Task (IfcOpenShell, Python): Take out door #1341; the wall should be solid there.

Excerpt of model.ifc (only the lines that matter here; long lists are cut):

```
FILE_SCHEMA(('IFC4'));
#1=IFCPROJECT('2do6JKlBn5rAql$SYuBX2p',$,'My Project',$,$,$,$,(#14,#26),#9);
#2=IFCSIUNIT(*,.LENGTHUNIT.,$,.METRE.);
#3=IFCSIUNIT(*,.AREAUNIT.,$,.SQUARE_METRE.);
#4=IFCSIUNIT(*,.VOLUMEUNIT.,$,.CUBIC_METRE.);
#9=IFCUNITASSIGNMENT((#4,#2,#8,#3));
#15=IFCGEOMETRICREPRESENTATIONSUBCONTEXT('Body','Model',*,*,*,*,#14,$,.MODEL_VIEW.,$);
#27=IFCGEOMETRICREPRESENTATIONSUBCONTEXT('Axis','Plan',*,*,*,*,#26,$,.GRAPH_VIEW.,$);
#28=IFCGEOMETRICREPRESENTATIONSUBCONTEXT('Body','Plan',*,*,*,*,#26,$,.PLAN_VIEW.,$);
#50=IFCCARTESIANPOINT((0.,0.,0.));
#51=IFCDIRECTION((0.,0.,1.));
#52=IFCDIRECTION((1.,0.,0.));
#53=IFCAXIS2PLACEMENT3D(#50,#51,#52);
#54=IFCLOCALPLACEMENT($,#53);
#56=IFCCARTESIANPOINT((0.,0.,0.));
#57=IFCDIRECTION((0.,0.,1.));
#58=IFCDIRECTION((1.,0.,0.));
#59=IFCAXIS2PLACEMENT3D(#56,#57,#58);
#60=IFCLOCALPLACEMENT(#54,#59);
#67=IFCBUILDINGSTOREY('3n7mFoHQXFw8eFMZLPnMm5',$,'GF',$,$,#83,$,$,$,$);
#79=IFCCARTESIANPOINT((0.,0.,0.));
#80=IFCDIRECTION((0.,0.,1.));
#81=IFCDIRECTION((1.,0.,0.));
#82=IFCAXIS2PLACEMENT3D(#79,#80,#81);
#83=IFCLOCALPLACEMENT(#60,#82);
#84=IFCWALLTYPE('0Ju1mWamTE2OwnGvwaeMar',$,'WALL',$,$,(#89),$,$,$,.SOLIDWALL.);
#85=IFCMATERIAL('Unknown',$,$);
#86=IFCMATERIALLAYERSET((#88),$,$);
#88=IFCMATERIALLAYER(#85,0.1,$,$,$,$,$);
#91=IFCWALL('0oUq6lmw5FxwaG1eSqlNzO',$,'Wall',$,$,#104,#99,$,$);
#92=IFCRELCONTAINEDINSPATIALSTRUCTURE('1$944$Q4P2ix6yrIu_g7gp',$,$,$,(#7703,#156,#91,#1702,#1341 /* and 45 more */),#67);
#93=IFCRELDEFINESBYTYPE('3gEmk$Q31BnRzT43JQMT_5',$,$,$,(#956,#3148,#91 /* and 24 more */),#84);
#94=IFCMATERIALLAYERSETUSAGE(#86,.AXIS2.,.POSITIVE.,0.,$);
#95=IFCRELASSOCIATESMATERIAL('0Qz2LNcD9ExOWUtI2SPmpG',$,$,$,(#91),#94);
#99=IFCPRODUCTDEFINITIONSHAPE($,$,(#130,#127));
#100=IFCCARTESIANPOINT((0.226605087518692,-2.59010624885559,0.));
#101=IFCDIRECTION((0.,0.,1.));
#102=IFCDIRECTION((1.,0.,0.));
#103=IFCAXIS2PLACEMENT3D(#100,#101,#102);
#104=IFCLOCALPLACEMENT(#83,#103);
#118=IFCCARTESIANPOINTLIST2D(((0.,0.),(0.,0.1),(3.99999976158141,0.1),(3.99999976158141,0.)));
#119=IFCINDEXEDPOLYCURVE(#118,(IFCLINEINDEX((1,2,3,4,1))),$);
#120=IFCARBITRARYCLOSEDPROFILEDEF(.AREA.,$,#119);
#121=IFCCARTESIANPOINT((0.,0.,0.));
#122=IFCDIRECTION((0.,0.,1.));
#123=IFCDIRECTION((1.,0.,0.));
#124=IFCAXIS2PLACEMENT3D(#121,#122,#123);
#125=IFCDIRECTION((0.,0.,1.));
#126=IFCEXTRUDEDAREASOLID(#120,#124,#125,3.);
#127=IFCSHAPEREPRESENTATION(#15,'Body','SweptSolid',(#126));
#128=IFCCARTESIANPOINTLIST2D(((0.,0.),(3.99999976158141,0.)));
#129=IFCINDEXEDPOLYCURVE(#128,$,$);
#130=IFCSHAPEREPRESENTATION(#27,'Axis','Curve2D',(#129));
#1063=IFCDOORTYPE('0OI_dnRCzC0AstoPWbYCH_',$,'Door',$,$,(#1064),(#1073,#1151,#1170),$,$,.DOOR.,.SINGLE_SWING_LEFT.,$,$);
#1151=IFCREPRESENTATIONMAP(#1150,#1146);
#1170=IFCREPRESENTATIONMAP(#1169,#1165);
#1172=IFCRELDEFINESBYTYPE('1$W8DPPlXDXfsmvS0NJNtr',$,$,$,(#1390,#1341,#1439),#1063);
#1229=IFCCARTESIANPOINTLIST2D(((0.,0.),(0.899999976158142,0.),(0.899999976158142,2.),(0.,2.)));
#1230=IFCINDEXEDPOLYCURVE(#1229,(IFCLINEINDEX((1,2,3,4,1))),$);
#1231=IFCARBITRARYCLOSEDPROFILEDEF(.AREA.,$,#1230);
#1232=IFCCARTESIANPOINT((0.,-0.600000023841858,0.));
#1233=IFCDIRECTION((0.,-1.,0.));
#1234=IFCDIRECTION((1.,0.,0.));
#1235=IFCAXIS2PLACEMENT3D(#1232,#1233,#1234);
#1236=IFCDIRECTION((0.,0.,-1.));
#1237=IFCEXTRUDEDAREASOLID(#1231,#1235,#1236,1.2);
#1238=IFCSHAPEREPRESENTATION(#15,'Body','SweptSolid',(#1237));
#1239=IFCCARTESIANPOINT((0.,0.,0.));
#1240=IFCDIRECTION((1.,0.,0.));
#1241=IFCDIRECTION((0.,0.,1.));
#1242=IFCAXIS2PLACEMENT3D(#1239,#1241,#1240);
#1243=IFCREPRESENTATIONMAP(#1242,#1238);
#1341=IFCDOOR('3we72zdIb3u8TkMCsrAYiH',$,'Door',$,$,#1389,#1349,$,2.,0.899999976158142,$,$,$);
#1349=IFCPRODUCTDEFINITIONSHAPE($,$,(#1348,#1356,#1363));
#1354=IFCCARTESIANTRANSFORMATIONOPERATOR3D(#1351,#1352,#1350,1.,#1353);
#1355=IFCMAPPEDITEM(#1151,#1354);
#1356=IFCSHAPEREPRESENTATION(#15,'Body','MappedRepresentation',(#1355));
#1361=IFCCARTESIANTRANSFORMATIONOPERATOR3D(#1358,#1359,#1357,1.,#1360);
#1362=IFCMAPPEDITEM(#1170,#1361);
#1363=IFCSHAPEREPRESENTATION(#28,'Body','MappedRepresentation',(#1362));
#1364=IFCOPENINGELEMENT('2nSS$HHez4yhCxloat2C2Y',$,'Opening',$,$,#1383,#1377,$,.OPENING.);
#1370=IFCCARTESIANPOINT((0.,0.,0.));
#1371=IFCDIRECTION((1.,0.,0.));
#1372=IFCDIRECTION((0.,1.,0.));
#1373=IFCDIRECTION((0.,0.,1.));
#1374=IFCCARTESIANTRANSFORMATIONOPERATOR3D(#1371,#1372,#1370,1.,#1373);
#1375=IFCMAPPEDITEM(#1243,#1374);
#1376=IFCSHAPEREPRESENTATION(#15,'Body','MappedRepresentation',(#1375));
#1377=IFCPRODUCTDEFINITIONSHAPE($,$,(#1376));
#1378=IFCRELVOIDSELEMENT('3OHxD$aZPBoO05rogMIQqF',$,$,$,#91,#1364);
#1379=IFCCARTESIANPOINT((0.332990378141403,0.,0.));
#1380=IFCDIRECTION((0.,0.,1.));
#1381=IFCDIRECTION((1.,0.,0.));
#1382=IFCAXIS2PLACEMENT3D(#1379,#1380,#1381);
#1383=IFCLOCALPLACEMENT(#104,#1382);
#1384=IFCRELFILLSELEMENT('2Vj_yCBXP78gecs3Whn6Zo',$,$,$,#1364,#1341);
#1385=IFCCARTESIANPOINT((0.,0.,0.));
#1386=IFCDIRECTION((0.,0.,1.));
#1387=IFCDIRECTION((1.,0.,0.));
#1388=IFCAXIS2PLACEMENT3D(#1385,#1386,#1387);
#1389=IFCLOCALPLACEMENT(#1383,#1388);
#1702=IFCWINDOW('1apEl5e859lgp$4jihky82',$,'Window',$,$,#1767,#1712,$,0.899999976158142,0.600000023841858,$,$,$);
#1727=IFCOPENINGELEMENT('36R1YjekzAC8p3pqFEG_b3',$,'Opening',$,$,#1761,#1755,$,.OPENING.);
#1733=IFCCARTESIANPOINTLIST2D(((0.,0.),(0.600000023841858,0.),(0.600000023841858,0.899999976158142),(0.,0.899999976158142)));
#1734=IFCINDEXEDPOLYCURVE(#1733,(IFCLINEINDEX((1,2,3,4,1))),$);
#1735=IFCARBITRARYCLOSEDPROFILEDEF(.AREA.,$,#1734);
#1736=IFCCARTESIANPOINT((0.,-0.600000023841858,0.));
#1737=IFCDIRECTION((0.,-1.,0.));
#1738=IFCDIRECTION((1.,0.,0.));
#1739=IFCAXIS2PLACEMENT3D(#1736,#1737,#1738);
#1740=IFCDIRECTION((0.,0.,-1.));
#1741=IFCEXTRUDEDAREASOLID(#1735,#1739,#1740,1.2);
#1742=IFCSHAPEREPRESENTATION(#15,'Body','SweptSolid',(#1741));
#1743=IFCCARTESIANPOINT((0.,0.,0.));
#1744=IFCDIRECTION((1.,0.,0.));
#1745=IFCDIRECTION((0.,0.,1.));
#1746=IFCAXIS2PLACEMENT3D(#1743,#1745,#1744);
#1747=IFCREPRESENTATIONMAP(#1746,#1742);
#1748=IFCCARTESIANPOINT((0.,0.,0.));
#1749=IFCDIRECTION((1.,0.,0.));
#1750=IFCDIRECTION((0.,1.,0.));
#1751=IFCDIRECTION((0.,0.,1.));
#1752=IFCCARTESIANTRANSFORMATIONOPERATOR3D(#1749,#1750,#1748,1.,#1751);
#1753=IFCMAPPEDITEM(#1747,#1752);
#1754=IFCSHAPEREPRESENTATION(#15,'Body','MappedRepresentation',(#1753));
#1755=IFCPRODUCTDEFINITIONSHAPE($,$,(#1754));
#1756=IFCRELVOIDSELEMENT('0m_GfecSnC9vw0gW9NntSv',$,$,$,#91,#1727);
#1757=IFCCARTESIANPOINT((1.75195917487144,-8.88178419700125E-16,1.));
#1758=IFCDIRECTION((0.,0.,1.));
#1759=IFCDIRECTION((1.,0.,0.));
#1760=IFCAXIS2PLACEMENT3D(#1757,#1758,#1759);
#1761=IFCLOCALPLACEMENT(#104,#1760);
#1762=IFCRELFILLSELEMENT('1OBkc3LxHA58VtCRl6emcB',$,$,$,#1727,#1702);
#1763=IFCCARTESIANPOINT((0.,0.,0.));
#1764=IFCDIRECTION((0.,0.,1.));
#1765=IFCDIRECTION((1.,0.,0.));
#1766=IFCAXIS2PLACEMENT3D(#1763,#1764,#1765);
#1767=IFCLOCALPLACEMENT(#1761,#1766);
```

```python
import ifcopenshell
import ifcopenshell.api.feature
import ifcopenshell.api.root
import ifcopenshell.geom
import ifcopenshell.util.shape

model = ifcopenshell.open("model.ifc")
settings = ifcopenshell.geom.settings()


def volume(element):
    """Net volume in cubic metres, openings subtracted."""
    shape = ifcopenshell.geom.create_shape(settings, element)
    return ifcopenshell.util.shape.get_volume(shape.geometry)


door = model.by_id(1341)
opening = door.FillsVoids[0].RelatingOpeningElement
wall = opening.VoidsElements[0].RelatingBuildingElement
before = volume(wall)

ifcopenshell.api.root.remove_product(model, product=door)
ifcopenshell.api.feature.remove_feature(model, feature=opening)

after = volume(wall)

print(f"wall volume {before:.3f} -> {after:.3f} m3")

model.write("model_rev.ifc")
```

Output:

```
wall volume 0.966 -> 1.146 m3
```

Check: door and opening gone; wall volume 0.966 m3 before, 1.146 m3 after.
